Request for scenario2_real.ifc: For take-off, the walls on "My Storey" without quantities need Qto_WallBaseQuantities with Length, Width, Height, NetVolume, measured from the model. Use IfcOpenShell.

First a look at what the model holds.

```python
import ifcopenshell
import ifcopenshell.util.element
import ifcopenshell.util.unit

model = ifcopenshell.open("scenario2_real.ifc")
print(model.schema)
for unit_type in ("LENGTHUNIT", "AREAUNIT", "VOLUMEUNIT"):
    print(unit_type, ifcopenshell.util.unit.calculate_unit_scale(model, unit_type))
storey = next(s for s in model.by_type("IfcBuildingStorey") if s.Name == "My Storey")
walls = [e for e in ifcopenshell.util.element.get_decomposition(storey) if e.is_a("IfcWall")]
for e in sorted(walls, key=lambda e: e.id()):
    print(e.id(), e.is_a(), e.Name, list(ifcopenshell.util.element.get_psets(e, qtos_only=True)), sep=" | ")
```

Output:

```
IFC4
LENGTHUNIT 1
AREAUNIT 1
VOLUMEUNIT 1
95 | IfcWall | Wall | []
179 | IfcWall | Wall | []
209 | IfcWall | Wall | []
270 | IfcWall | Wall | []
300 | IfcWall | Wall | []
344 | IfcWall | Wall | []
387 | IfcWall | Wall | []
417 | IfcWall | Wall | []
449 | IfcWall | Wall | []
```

```python
import ifcopenshell
import ifcopenshell.api.pset
import ifcopenshell.geom
import ifcopenshell.util.element
import ifcopenshell.util.shape
import ifcopenshell.util.unit

model = ifcopenshell.open("scenario2_real.ifc")
unit_scale = ifcopenshell.util.unit.calculate_unit_scale(model)
volume_scale = ifcopenshell.util.unit.calculate_unit_scale(model, "VOLUMEUNIT")
settings = ifcopenshell.geom.settings()

storey = next(s for s in model.by_type("IfcBuildingStorey") if s.Name == "My Storey")
walls = [e for e in ifcopenshell.util.element.get_decomposition(storey) if e.is_a("IfcWall")]

for e in sorted(walls, key=lambda e: e.id()):
    if ifcopenshell.util.element.get_psets(e, qtos_only=True, should_inherit=False):
        continue
    # Geometry comes back in metres, in the element's own axes.
    shape = ifcopenshell.geom.create_shape(settings, e)
    values = {
        "Length": ifcopenshell.util.shape.get_x(shape.geometry) / unit_scale,
        "Width": ifcopenshell.util.shape.get_y(shape.geometry) / unit_scale,
        "Height": ifcopenshell.util.shape.get_z(shape.geometry) / unit_scale,
        "NetVolume": ifcopenshell.util.shape.get_volume(shape.geometry) / volume_scale,
    }
    qto = ifcopenshell.api.pset.add_qto(model, product=e, name="Qto_WallBaseQuantities")
    ifcopenshell.api.pset.edit_qto(model, qto=qto, properties=values)
    print(e.id(), {k: round(v, 3) for k, v in values.items()})

model.write("scenario2_real_edited.ifc")
```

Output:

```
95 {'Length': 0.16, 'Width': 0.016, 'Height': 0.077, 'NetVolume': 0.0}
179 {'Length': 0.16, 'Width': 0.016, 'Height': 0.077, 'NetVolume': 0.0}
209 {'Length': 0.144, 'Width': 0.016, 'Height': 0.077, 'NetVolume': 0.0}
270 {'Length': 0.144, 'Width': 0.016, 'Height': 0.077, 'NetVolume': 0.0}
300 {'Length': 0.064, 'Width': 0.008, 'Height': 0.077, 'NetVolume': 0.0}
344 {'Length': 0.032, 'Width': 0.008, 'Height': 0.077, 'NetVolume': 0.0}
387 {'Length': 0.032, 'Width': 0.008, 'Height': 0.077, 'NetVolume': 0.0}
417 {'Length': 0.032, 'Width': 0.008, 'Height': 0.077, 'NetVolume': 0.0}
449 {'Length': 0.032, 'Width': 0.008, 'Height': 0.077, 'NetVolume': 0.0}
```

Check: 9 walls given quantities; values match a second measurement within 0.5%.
